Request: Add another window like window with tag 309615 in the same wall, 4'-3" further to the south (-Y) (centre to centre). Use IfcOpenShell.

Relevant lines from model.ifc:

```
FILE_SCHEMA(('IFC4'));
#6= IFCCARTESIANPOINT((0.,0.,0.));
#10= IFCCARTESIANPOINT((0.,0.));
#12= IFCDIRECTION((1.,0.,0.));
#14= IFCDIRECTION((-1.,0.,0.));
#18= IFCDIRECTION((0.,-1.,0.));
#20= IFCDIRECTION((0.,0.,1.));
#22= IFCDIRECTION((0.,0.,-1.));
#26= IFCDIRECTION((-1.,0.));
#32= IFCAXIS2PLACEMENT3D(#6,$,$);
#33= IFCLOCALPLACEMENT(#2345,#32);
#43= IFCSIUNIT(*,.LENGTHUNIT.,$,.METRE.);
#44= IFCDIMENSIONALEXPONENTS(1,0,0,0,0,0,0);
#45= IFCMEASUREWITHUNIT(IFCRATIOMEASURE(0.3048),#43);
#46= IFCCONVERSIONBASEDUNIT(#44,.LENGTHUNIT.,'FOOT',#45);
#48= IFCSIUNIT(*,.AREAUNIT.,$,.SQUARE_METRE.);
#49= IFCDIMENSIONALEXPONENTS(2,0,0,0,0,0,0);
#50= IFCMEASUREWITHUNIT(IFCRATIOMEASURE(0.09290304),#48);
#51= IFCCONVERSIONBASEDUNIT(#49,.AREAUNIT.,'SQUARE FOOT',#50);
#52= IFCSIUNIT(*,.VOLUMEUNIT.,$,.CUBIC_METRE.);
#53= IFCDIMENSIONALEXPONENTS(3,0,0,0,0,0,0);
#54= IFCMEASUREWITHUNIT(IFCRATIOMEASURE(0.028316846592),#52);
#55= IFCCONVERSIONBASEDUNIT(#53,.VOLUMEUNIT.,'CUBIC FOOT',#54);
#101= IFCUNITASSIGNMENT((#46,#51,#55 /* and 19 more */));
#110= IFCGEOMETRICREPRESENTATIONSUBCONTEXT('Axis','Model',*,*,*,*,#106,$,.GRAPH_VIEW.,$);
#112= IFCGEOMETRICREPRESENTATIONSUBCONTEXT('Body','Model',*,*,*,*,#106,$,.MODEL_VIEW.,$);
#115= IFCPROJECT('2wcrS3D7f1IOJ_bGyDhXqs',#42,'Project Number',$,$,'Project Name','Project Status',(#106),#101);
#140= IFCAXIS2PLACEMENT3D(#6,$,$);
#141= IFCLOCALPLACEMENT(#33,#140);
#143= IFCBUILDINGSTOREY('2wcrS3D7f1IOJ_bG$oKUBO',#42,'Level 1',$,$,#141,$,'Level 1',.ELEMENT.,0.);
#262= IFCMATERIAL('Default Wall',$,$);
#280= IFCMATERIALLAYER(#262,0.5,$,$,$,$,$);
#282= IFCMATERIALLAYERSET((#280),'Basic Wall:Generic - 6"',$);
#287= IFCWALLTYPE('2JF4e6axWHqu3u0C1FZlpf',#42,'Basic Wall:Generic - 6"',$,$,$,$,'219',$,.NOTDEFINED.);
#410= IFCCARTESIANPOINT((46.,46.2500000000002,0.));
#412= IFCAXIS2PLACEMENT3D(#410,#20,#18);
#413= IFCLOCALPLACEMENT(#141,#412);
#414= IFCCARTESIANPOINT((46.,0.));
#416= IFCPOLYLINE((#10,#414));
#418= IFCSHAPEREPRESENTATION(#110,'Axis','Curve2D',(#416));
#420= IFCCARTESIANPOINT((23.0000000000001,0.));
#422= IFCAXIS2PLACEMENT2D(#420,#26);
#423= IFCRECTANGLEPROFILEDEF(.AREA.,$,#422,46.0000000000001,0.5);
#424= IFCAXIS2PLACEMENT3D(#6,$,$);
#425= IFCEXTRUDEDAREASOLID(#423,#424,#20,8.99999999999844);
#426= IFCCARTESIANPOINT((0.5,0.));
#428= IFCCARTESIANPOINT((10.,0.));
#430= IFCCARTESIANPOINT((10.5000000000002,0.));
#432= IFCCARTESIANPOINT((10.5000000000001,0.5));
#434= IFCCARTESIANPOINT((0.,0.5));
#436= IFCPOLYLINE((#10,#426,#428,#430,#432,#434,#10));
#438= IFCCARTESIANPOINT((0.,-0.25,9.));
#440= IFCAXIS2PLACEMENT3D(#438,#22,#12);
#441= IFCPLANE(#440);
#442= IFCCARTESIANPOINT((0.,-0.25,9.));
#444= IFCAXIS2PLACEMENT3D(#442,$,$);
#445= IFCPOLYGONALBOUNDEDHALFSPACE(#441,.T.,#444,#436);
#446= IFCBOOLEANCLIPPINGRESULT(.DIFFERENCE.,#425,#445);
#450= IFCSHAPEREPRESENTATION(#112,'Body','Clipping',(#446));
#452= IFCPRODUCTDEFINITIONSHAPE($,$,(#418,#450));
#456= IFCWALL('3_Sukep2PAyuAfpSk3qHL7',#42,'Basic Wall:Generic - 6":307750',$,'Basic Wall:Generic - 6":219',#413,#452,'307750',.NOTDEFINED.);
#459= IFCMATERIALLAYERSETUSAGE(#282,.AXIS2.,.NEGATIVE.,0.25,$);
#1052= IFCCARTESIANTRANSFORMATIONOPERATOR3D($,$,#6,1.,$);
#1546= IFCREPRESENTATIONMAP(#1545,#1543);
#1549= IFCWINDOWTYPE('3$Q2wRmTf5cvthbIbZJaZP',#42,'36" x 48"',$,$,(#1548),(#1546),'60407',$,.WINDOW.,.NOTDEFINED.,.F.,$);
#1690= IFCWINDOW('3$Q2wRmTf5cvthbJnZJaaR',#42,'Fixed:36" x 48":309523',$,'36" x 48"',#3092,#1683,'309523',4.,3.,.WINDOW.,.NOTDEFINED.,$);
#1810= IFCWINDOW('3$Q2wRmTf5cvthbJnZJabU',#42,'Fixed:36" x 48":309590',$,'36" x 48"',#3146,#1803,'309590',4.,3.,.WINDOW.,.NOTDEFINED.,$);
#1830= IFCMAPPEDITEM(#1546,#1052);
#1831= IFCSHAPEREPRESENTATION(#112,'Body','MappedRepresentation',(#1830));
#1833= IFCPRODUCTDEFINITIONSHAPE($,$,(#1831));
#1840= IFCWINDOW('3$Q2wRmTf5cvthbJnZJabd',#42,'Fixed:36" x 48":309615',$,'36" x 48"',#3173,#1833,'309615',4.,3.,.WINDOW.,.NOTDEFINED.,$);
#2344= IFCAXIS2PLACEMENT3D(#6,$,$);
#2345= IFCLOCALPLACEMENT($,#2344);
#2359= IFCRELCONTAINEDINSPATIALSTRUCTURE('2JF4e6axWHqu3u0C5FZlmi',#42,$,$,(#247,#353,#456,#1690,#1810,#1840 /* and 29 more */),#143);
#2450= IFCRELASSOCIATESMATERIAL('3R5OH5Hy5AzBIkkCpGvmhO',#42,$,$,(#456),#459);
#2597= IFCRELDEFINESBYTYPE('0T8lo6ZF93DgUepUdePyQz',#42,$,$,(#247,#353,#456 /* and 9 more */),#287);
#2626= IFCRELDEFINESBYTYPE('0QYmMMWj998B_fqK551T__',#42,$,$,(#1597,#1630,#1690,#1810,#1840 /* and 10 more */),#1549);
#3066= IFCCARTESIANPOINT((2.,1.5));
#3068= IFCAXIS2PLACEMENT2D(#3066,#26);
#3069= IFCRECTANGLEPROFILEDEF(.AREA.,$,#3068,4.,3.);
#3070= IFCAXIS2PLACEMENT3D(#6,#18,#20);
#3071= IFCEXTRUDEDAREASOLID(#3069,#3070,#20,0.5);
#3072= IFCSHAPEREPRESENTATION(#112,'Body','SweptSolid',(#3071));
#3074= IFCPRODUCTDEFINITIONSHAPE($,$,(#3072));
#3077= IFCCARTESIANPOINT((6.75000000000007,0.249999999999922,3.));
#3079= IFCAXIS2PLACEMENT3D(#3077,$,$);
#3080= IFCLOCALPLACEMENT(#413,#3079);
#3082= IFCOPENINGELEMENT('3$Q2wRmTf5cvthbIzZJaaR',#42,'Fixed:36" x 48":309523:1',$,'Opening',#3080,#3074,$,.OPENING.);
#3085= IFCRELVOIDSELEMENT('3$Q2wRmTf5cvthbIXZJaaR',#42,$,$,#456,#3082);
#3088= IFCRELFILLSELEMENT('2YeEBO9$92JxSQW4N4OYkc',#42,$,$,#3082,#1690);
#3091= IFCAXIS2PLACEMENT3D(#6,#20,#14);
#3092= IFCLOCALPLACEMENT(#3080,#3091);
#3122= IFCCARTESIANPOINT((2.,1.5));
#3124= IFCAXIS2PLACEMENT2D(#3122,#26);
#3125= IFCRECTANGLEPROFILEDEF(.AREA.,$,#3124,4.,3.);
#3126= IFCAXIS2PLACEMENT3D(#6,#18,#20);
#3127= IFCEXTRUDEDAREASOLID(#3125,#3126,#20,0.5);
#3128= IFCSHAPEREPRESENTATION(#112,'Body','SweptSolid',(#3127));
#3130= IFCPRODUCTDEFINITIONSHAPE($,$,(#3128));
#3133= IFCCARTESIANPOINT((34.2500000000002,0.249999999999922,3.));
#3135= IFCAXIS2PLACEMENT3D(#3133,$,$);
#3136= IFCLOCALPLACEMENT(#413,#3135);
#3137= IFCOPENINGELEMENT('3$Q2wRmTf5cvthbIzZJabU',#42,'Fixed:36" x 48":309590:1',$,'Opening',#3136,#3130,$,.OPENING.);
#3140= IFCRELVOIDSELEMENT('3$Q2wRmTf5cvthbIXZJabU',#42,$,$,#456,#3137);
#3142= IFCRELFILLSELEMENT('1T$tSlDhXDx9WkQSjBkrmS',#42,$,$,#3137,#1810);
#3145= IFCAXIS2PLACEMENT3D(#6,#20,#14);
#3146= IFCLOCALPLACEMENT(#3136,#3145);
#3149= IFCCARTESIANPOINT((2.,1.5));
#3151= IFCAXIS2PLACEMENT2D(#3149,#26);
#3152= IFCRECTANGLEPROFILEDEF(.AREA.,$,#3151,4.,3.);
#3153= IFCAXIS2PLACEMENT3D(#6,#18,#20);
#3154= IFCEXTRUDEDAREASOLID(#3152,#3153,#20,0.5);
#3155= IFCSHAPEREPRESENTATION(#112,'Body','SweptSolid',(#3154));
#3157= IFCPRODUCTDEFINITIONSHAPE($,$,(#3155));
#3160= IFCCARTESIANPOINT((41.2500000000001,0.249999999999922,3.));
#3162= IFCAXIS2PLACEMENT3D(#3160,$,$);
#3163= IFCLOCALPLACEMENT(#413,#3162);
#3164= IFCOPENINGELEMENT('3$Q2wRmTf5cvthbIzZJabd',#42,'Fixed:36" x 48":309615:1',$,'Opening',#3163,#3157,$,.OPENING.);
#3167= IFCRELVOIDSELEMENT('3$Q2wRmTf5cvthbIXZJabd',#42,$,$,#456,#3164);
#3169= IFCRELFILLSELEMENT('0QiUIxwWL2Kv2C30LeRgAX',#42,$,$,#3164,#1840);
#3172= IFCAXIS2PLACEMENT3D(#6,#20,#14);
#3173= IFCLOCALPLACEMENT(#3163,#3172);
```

```python
import ifcopenshell
import ifcopenshell.api.feature
import ifcopenshell.api.geometry
import ifcopenshell.api.root
import ifcopenshell.geom
import ifcopenshell.util.element
import ifcopenshell.util.placement
import ifcopenshell.util.shape
import ifcopenshell.util.unit

model = ifcopenshell.open("model.ifc")
unit_scale = ifcopenshell.util.unit.calculate_unit_scale(model)
settings = ifcopenshell.geom.settings()


def volume(element):
    """Net volume in cubic metres, openings subtracted."""
    shape = ifcopenshell.geom.create_shape(settings, element)
    return ifcopenshell.util.shape.get_volume(shape.geometry)


def reuse_history(source, copy):
    """copy_class also copies each property set's owner history, people and application; keep the originals."""
    for rel in copy.IsDefinedBy:
        if rel.is_a("IfcRelDefinesByProperties") and (history := rel.RelatingPropertyDefinition.OwnerHistory):
            rel.RelatingPropertyDefinition.OwnerHistory = source.OwnerHistory
            ifcopenshell.util.element.remove_deep2(model, history)


window = model.by_guid("3$Q2wRmTf5cvthbJnZJabd")
opening = window.FillsVoids[0].RelatingOpeningElement
wall = opening.VoidsElements[0].RelatingBuildingElement
before = volume(wall)
shift = ifcopenshell.util.placement.get_local_placement(wall.ObjectPlacement)[:3, 0] * 51 * 0.0254 / unit_scale

# copy_class copies the void relationship, type, container and properties, but no geometry.
new_opening = ifcopenshell.api.root.copy_class(model, product=opening)
new_opening.Representation = ifcopenshell.util.element.copy_deep(
    model, opening.Representation, exclude=["IfcGeometricRepresentationContext", "IfcRepresentationMap"]
)
new_opening.Name = 'Fixed:36" x 48"'
new_window = ifcopenshell.api.root.copy_class(model, product=window)
new_window.Representation = ifcopenshell.util.element.copy_deep(
    model, window.Representation, exclude=["IfcGeometricRepresentationContext", "IfcRepresentationMap"]
)
new_window.Name = 'Fixed:36" x 48"'
new_window.Tag = None
reuse_history(window, new_window)
ifcopenshell.api.feature.add_filling(model, opening=new_opening, element=new_window)

for old, new in ((opening, new_opening), (window, new_window)):
    matrix = ifcopenshell.util.placement.get_local_placement(old.ObjectPlacement)
    matrix[:3, 3] += shift
    ifcopenshell.api.geometry.edit_object_placement(model, product=new, matrix=matrix, is_si=False)

after = volume(wall)

print(f"wall volume {before:.3f} -> {after:.3f} m3")

model.write("model_rev.ifc")
```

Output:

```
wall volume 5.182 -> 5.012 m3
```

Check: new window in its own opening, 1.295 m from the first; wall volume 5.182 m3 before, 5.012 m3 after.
